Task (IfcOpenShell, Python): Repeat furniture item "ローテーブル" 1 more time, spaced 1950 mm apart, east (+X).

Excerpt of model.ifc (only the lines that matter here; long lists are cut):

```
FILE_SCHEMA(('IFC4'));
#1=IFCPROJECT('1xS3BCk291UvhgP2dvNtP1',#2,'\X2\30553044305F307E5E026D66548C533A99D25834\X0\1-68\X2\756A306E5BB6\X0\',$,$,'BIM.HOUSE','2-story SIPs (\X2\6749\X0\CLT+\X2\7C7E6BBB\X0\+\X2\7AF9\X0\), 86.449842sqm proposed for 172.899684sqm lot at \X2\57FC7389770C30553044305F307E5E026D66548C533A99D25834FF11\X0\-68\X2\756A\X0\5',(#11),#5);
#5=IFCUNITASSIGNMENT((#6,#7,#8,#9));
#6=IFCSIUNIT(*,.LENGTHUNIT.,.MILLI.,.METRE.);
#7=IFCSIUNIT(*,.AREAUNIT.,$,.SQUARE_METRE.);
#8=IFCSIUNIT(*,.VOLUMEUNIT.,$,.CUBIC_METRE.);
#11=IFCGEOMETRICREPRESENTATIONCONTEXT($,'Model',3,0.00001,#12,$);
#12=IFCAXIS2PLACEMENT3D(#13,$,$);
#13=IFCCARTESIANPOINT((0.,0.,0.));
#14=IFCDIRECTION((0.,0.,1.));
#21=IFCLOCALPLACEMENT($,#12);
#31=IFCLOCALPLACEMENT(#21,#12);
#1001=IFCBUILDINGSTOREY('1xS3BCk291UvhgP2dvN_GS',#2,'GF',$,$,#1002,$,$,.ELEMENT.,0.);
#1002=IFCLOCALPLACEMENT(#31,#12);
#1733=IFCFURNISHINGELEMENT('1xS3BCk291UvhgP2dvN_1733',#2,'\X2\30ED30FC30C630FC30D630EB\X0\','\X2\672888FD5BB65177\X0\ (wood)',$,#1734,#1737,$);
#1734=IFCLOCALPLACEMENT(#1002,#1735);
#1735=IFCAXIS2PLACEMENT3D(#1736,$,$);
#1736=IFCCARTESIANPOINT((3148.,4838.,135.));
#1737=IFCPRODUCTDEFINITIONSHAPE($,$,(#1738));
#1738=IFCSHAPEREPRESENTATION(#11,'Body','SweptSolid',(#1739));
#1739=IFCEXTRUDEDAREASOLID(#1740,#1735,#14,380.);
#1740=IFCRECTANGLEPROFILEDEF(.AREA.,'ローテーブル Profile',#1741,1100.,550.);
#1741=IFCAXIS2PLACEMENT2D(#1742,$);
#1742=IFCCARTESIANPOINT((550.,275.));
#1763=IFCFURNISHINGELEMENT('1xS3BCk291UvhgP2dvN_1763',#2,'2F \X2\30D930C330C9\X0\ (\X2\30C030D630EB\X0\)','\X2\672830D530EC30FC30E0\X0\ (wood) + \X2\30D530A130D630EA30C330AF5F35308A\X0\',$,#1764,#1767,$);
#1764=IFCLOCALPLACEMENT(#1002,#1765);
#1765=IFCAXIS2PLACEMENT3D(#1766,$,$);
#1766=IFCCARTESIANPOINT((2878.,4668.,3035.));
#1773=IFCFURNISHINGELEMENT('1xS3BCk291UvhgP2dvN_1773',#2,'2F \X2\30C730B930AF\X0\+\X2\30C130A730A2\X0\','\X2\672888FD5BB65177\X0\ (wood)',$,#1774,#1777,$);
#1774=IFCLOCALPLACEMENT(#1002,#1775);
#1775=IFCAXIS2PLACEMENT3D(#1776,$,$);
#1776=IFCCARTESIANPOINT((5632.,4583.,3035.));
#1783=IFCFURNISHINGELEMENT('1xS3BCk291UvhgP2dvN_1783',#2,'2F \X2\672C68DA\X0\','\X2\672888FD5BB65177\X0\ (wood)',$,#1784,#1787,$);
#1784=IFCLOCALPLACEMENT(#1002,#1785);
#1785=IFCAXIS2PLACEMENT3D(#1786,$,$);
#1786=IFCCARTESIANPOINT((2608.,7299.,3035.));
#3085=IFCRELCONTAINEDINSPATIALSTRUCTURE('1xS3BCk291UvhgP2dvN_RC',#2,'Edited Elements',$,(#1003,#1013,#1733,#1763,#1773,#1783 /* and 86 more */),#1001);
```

```python
import numpy as np
import ifcopenshell
import ifcopenshell.api.geometry
import ifcopenshell.api.root
import ifcopenshell.util.element
import ifcopenshell.util.placement
import ifcopenshell.util.unit

model = ifcopenshell.open("model.ifc")
unit_scale = ifcopenshell.util.unit.calculate_unit_scale(model)


def reuse_history(source, copy):
    """copy_class also copies each property set's owner history, people and application; keep the originals."""
    for rel in copy.IsDefinedBy:
        if rel.is_a("IfcRelDefinesByProperties") and (history := rel.RelatingPropertyDefinition.OwnerHistory):
            rel.RelatingPropertyDefinition.OwnerHistory = source.OwnerHistory
            ifcopenshell.util.element.remove_deep2(model, history)


source = model.by_guid("1xS3BCk291UvhgP2dvN_1733")
base = ifcopenshell.util.placement.get_local_placement(source.ObjectPlacement)
step = np.array([1.0, 0.0, 0.0]) * 1.95 / unit_scale

for i in range(1, 2):
    copy = ifcopenshell.api.root.copy_class(model, product=source)
    copy.Representation = ifcopenshell.util.element.copy_deep(
        model, source.Representation, exclude=["IfcGeometricRepresentationContext", "IfcRepresentationMap"]
    )
    reuse_history(source, copy)
    matrix = base.copy()
    matrix[:3, 3] += i * step
    print("added at", matrix[:3, 3].round(3) + 0.0)
    ifcopenshell.api.geometry.edit_object_placement(model, product=copy, matrix=matrix, is_si=False)

model.write("model_v2.ifc")
```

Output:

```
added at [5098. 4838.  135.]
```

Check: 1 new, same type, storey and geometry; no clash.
